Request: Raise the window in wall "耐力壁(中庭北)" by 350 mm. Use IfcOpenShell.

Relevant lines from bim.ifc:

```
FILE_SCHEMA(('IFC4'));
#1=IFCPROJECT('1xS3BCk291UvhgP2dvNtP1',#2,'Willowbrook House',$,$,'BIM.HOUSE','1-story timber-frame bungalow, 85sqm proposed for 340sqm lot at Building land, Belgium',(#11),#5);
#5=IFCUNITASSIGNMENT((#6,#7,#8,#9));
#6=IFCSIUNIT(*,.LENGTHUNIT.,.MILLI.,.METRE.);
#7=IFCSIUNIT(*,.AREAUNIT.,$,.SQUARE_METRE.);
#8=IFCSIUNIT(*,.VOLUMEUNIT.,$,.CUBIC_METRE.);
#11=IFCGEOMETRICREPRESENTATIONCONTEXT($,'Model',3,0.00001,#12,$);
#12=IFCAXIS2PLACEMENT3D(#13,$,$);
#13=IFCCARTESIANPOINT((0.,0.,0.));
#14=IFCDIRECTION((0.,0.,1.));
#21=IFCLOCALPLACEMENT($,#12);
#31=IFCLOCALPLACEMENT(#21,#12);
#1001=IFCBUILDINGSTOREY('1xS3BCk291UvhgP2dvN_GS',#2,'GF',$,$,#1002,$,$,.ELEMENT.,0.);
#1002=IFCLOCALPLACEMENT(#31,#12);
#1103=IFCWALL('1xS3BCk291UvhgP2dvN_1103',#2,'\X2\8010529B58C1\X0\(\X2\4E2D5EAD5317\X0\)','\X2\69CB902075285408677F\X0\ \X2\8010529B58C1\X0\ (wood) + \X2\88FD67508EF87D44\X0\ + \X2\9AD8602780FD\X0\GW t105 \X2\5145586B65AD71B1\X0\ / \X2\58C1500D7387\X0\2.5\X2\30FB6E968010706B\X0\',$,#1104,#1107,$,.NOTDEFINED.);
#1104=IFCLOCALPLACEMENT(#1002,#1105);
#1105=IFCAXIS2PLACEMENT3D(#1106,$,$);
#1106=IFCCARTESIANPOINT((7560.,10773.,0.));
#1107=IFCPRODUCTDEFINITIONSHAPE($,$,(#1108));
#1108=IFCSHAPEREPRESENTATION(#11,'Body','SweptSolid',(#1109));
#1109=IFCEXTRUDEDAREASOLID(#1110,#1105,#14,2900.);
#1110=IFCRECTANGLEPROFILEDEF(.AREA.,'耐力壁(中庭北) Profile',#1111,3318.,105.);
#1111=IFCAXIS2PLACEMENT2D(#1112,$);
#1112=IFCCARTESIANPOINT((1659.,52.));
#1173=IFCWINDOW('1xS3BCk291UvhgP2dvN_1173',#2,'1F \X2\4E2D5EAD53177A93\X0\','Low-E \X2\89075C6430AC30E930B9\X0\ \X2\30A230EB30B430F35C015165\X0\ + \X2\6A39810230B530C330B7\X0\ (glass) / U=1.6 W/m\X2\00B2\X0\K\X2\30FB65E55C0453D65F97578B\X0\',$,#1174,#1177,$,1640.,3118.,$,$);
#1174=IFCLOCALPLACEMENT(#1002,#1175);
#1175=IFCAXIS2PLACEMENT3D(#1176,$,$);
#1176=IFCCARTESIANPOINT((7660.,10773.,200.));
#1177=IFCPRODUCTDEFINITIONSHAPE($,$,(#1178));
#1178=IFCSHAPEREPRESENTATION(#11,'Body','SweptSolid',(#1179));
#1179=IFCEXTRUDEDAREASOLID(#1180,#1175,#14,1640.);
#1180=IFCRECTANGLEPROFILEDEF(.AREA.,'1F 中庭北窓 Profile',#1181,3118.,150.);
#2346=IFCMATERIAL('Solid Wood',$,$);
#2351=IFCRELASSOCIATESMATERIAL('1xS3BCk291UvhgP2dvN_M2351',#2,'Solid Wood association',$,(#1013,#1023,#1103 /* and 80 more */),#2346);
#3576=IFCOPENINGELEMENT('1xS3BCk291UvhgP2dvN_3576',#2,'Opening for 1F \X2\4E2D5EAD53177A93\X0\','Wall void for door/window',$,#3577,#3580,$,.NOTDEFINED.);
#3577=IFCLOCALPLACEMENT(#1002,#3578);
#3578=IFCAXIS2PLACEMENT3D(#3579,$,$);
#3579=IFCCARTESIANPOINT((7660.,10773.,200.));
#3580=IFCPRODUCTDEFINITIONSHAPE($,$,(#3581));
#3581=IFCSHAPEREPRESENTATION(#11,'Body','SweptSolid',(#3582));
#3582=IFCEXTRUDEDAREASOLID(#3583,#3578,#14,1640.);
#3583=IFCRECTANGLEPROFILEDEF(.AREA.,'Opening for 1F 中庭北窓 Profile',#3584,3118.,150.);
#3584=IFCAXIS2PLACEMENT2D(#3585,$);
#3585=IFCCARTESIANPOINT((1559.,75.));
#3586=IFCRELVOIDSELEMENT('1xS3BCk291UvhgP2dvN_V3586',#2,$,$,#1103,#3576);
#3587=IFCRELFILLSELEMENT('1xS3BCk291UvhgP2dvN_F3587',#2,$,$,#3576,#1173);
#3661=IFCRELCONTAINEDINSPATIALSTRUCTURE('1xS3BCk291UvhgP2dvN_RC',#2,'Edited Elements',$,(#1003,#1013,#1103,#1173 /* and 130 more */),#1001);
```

```python
import numpy as np
import ifcopenshell
import ifcopenshell.api.geometry
import ifcopenshell.util.placement
import ifcopenshell.util.unit

model = ifcopenshell.open("bim.ifc")
unit_scale = ifcopenshell.util.unit.calculate_unit_scale(model)

window = model.by_id(1173)
opening = window.FillsVoids[0].RelatingOpeningElement
dz = 0.35 / unit_scale

shift = np.array([0.0, 0.0, dz])
# The window is not placed relative to its opening, so move both.
for product in (opening, window):
    matrix = ifcopenshell.util.placement.get_local_placement(product.ObjectPlacement)
    matrix[:3, 3] += shift
    ifcopenshell.api.geometry.edit_object_placement(model, product=product, matrix=matrix, is_si=False)

print(f"moved by {dz * unit_scale:+.3f} m")

model.write("bim_updated.ifc")
```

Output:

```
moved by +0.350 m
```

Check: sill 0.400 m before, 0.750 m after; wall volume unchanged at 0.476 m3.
